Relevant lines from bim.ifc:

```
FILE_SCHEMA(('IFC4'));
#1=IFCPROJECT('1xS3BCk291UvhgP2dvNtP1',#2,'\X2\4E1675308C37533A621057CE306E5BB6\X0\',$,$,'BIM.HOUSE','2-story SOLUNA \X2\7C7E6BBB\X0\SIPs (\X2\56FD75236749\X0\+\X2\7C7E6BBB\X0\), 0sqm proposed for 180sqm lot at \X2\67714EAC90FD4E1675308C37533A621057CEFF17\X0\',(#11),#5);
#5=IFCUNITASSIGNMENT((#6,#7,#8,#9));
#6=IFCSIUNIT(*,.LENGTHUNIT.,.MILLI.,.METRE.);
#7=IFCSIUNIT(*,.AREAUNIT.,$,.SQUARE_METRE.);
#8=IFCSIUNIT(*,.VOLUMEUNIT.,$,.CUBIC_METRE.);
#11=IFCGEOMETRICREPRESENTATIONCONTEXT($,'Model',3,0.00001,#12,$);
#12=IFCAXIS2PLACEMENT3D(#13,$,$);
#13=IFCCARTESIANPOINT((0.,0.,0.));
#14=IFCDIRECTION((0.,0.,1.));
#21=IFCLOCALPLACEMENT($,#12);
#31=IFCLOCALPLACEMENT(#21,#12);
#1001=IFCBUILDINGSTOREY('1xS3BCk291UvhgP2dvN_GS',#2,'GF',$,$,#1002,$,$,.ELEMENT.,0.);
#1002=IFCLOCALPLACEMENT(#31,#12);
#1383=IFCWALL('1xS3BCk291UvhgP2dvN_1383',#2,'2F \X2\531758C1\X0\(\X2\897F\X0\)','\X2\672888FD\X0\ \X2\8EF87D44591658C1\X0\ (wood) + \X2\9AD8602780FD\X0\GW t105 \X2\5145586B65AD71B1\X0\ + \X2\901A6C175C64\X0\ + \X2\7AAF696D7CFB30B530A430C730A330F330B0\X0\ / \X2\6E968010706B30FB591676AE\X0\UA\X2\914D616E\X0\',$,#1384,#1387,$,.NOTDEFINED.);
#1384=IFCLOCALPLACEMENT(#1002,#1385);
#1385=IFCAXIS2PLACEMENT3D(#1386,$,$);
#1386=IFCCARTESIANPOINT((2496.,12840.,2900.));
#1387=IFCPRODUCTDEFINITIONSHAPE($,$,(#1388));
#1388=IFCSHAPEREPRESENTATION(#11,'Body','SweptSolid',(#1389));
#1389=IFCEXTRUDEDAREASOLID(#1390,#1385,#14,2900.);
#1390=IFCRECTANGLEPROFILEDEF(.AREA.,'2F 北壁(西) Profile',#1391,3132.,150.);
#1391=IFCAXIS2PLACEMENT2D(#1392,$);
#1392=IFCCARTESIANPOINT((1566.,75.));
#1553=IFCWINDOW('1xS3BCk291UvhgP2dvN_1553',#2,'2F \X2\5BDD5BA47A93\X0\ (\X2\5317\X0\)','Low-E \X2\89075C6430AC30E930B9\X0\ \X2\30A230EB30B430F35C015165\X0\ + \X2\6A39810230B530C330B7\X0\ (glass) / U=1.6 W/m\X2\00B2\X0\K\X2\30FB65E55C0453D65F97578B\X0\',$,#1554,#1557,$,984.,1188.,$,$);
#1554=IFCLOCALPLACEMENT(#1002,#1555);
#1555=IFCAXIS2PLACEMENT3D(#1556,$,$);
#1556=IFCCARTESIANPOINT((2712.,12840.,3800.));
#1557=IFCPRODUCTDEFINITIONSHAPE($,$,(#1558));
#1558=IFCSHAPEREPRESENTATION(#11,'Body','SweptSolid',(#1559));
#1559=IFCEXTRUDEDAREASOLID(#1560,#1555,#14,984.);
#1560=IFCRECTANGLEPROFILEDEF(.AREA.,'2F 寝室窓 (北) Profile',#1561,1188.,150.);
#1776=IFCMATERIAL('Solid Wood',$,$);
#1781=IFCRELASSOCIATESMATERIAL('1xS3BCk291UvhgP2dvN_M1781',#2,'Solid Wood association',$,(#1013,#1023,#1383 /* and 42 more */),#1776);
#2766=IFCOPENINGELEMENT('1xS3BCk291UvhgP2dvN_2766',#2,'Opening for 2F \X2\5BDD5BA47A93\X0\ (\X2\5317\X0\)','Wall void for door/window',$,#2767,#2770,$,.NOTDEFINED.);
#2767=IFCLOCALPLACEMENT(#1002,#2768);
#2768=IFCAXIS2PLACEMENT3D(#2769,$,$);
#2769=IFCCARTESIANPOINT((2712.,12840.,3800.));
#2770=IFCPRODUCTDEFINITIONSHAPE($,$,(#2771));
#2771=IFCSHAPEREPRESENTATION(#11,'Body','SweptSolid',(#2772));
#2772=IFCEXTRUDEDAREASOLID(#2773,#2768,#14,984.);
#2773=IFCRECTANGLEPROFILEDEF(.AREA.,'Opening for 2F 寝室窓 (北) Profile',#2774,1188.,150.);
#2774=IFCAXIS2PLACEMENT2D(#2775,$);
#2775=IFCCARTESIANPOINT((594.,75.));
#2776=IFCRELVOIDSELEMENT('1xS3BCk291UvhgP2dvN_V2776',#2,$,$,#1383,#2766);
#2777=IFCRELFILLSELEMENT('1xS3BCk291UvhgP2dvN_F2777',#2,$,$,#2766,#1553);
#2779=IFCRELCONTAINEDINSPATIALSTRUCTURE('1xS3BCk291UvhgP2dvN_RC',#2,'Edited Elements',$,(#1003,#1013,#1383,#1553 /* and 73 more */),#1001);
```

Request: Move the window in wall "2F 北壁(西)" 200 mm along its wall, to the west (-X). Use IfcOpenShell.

```python
import ifcopenshell
import ifcopenshell.api.geometry
import ifcopenshell.util.placement

model = ifcopenshell.open("bim.ifc")

window = model.by_guid("1xS3BCk291UvhgP2dvN_1553")
opening = window.FillsVoids[0].RelatingOpeningElement
wall = opening.VoidsElements[0].RelatingBuildingElement

wall_matrix = ifcopenshell.util.placement.get_local_placement(wall.ObjectPlacement)
shift = wall_matrix[:3, 0] * -200.0
before = ifcopenshell.util.placement.get_local_placement(window.ObjectPlacement)[:3, 3].copy()

# The window is not placed relative to its opening, so move both.
for product in (opening, window):
    matrix = ifcopenshell.util.placement.get_local_placement(product.ObjectPlacement)
    matrix[:3, 3] += shift
    ifcopenshell.api.geometry.edit_object_placement(model, product=product, matrix=matrix, is_si=False)

after = ifcopenshell.util.placement.get_local_placement(window.ObjectPlacement)[:3, 3]
print("window moved by", (after - before).round(3) + 0.0)

model.write("bim-out.ifc")
```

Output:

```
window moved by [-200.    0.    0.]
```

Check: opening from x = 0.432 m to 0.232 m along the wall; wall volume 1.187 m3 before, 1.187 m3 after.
